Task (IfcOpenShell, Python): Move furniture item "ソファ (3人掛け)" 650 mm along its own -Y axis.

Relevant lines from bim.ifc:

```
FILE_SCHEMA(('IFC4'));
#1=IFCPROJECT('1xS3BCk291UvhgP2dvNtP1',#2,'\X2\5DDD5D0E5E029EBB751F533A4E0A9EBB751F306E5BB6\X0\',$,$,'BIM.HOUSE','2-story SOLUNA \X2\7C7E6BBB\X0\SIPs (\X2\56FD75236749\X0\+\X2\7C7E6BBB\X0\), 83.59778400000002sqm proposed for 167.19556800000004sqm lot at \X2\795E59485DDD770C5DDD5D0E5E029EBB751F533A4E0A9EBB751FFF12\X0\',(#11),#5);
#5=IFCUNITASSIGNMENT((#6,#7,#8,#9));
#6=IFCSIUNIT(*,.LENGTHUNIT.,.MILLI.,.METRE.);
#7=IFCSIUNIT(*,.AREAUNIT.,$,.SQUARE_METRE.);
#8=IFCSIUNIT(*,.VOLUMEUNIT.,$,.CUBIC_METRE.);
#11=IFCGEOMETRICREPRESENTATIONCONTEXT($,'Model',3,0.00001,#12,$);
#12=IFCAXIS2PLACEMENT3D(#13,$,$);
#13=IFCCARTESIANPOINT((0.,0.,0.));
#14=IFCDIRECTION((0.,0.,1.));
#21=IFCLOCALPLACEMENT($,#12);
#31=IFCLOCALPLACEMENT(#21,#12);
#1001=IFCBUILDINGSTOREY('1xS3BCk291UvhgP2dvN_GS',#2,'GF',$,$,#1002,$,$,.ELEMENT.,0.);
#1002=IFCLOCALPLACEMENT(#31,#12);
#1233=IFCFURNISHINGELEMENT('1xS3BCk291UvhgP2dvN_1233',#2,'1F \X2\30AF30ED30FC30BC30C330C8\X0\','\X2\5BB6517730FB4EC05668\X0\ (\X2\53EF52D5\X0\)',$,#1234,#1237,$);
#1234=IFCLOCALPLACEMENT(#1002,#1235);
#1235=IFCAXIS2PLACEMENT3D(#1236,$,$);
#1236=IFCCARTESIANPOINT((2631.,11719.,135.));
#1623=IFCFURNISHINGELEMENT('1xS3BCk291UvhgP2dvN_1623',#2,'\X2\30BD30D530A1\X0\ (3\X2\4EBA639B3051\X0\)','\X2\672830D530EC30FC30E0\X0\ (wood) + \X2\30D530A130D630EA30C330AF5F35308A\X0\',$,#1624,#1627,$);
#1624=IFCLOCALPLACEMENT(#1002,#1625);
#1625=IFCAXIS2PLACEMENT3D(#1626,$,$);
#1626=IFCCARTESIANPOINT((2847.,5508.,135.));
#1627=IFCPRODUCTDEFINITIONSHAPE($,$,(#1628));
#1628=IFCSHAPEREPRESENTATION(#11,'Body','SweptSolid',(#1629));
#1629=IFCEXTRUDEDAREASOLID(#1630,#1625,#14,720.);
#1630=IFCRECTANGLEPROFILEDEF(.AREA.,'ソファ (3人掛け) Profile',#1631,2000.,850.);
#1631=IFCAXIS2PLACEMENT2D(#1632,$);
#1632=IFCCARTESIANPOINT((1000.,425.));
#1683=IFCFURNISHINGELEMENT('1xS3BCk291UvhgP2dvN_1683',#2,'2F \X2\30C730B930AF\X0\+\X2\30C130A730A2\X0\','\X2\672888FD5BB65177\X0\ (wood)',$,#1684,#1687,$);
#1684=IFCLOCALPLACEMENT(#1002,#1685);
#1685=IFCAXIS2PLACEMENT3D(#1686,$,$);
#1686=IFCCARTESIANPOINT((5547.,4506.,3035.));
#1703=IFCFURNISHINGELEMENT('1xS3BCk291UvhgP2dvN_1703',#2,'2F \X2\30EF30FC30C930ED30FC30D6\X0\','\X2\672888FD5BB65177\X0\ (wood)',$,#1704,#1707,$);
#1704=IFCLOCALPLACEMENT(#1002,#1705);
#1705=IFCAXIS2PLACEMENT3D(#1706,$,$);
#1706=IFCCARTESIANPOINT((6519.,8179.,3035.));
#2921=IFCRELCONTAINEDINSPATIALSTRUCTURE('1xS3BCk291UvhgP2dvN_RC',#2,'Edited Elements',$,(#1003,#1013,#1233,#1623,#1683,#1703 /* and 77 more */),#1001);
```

```python
import ifcopenshell
import ifcopenshell.api.geometry
import ifcopenshell.util.placement
import ifcopenshell.util.unit

model = ifcopenshell.open("bim.ifc")
unit_scale = ifcopenshell.util.unit.calculate_unit_scale(model)

item = model.by_guid("1xS3BCk291UvhgP2dvN_1623")
matrix = ifcopenshell.util.placement.get_local_placement(item.ObjectPlacement)
matrix[:3, 3] -= matrix[:3, 1] * 0.65 / unit_scale
ifcopenshell.api.geometry.edit_object_placement(model, product=item, matrix=matrix, is_si=False)

print(ifcopenshell.util.placement.get_local_placement(item.ObjectPlacement).round(3) + 0.0)

model.write("bim-out.ifc")
```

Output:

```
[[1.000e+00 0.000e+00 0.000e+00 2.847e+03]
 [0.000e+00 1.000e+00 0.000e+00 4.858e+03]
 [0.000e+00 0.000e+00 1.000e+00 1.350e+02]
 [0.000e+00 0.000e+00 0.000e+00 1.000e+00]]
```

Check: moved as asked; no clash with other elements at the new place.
